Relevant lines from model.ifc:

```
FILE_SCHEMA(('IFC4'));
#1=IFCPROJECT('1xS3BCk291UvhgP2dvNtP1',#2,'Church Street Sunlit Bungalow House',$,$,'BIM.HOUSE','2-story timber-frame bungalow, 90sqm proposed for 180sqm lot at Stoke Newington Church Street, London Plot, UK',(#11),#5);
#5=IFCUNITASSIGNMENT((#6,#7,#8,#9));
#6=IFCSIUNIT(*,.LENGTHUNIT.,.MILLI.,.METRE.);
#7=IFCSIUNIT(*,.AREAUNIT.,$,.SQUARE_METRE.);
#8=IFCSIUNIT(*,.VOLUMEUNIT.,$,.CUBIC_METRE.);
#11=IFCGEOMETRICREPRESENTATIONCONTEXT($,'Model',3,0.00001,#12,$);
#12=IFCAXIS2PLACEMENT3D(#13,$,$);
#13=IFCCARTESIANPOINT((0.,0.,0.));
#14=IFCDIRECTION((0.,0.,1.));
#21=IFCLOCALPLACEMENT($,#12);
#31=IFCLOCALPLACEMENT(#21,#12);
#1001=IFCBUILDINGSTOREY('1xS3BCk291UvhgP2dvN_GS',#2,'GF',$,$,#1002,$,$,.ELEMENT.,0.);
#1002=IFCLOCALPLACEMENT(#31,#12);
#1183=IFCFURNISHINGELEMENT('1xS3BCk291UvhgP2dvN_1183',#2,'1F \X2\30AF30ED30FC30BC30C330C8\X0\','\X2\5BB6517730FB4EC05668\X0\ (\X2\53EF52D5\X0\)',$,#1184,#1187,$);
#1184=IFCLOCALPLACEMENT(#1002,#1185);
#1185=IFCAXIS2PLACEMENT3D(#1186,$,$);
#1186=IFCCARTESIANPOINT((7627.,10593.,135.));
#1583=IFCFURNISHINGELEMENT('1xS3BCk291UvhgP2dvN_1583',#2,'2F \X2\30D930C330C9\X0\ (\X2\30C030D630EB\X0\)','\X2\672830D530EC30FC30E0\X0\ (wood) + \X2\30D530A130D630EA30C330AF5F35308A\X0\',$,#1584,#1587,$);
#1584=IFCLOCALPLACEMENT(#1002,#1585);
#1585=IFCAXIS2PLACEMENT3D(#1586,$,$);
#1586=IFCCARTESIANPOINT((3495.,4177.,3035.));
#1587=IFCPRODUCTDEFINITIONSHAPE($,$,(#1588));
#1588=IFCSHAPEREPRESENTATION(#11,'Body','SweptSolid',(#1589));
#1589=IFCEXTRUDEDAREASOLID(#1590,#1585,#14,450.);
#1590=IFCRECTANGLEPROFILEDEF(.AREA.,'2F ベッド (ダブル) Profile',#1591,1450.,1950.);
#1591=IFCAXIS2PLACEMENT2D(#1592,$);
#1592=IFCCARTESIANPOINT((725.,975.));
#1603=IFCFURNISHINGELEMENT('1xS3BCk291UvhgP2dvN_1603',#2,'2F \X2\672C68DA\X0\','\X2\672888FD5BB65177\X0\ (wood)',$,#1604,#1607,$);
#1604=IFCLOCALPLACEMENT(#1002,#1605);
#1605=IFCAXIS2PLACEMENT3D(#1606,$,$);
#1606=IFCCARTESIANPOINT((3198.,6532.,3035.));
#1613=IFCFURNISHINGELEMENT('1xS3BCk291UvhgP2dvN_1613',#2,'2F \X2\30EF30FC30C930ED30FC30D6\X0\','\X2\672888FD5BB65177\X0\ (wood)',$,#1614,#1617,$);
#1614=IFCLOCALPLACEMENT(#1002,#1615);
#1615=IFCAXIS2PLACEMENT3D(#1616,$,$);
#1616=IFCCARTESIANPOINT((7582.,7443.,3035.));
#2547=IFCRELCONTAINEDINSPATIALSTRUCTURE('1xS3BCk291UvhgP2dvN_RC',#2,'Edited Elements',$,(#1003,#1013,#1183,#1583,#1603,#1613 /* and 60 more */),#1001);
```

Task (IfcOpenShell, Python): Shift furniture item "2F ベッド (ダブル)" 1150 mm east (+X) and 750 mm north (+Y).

```python
import ifcopenshell
import ifcopenshell.api.geometry
import ifcopenshell.util.placement
import ifcopenshell.util.unit

model = ifcopenshell.open("model.ifc")
unit_scale = ifcopenshell.util.unit.calculate_unit_scale(model)

item = model.by_guid("1xS3BCk291UvhgP2dvN_1583")
matrix = ifcopenshell.util.placement.get_local_placement(item.ObjectPlacement)
matrix[0, 3] += 1.15 / unit_scale
matrix[1, 3] += 0.75 / unit_scale
ifcopenshell.api.geometry.edit_object_placement(model, product=item, matrix=matrix, is_si=False)

print(ifcopenshell.util.placement.get_local_placement(item.ObjectPlacement).round(3) + 0.0)

model.write("model_rev.ifc")
```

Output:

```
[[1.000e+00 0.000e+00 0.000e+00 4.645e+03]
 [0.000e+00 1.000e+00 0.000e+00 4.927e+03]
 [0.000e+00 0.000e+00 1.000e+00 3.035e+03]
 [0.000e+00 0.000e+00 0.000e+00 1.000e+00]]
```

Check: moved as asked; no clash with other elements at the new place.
